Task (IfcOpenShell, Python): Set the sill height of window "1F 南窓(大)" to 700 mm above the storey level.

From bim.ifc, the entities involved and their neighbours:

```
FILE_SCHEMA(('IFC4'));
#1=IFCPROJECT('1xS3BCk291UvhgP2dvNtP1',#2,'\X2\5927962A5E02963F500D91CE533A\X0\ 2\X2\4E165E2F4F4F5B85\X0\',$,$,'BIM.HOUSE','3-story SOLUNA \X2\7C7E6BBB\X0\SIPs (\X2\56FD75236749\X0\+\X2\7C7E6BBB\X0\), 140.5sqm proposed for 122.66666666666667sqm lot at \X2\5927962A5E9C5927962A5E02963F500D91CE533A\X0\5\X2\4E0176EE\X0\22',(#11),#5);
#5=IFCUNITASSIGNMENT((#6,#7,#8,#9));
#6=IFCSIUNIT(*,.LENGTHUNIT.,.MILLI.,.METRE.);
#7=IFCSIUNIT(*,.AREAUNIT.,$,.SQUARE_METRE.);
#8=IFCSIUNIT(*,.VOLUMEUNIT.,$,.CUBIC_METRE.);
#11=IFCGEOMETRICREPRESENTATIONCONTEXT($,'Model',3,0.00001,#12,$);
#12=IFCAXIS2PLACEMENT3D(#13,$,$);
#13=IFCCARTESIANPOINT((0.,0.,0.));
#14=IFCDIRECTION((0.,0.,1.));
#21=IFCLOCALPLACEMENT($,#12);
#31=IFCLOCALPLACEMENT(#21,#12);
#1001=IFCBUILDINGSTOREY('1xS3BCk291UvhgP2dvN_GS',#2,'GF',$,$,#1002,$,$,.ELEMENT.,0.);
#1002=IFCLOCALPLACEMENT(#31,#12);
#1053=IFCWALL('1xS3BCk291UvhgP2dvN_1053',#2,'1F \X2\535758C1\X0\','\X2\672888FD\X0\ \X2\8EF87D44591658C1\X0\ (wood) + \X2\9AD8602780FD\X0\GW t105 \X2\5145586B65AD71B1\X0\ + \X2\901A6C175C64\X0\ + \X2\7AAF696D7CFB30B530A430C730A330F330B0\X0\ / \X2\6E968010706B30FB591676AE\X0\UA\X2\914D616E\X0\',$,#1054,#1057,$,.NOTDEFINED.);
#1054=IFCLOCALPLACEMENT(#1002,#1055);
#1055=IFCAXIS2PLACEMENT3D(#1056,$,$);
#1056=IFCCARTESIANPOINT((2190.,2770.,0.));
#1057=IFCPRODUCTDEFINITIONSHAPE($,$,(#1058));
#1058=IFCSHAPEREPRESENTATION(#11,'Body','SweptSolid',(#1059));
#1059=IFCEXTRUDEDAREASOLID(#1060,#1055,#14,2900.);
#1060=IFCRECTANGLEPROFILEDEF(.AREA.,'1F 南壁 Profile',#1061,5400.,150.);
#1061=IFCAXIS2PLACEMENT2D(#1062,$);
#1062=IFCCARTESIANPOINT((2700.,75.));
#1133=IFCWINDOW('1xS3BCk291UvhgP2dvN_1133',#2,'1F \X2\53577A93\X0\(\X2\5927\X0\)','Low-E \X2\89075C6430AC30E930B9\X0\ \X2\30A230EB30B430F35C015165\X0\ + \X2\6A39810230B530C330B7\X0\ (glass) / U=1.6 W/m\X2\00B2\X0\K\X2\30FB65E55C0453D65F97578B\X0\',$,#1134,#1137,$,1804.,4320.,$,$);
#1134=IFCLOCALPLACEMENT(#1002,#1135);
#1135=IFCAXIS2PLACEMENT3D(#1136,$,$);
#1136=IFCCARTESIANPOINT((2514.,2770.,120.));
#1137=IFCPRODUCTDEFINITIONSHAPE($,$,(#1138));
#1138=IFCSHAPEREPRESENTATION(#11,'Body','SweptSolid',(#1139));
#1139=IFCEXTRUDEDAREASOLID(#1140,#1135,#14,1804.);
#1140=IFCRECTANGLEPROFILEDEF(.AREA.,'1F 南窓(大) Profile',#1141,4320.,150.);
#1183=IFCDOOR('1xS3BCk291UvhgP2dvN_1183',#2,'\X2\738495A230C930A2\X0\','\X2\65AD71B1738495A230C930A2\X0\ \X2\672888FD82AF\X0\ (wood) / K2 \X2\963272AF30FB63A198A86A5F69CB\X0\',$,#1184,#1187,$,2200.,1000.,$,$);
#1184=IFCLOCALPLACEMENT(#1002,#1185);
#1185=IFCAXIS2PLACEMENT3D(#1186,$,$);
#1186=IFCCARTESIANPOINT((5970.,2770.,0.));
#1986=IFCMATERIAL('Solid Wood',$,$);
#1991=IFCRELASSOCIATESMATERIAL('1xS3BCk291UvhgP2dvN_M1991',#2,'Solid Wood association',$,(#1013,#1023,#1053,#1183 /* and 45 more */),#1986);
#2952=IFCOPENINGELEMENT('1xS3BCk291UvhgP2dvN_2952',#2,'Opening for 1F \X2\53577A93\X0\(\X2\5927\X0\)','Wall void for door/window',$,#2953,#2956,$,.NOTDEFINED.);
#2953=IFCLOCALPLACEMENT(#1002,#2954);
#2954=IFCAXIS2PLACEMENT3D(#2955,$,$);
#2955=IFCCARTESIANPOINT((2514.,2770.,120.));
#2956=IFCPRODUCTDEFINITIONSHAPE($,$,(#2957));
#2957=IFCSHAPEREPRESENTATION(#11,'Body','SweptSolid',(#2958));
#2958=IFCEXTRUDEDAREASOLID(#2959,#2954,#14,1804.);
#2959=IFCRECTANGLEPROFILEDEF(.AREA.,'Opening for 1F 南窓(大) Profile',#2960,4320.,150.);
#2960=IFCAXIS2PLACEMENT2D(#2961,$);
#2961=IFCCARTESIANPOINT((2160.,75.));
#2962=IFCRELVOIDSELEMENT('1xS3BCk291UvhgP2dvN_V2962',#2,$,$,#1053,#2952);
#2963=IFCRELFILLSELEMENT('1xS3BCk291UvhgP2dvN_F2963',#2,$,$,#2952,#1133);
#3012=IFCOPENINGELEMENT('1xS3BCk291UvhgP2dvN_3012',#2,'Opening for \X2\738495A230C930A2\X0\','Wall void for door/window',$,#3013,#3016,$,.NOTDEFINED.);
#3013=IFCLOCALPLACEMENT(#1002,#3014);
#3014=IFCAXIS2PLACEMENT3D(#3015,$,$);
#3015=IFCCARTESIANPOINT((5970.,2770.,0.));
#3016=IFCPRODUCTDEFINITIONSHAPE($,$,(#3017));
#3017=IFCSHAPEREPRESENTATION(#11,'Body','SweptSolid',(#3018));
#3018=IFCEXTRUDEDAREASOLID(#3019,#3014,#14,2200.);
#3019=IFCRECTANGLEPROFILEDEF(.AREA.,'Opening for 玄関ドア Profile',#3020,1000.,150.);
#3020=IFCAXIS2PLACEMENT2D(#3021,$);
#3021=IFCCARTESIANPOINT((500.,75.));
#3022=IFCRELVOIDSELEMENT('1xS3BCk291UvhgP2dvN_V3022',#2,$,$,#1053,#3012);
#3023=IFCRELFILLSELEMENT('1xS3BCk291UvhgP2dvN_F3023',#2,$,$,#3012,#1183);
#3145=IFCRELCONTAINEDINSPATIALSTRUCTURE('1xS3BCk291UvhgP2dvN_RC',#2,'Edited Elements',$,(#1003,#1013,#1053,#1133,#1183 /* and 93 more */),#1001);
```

```python
import numpy as np
import ifcopenshell
import ifcopenshell.api.geometry
import ifcopenshell.geom
import ifcopenshell.util.element
import ifcopenshell.util.placement
import ifcopenshell.util.shape
import ifcopenshell.util.unit

model = ifcopenshell.open("bim.ifc")
unit_scale = ifcopenshell.util.unit.calculate_unit_scale(model)

window = model.by_guid("1xS3BCk291UvhgP2dvN_1133")
opening = window.FillsVoids[0].RelatingOpeningElement
storey = ifcopenshell.util.element.get_container(window, ifc_class="IfcBuildingStorey")
level = ifcopenshell.util.placement.get_local_placement(storey.ObjectPlacement)[2, 3]

# The opening's origin need not be at the sill, so measure its lowest point.
shape = ifcopenshell.geom.create_shape(ifcopenshell.geom.settings(), opening)
bottom = ifcopenshell.util.shape.get_shape_bottom_elevation(shape, shape.geometry) / unit_scale
dz = level + 0.7 / unit_scale - bottom

shift = np.array([0.0, 0.0, dz])
# The window is not placed relative to its opening, so move both.
for product in (opening, window):
    matrix = ifcopenshell.util.placement.get_local_placement(product.ObjectPlacement)
    matrix[:3, 3] += shift
    ifcopenshell.api.geometry.edit_object_placement(model, product=product, matrix=matrix, is_si=False)

print(f"moved by {dz * unit_scale:+.3f} m")

model.write("bim-out.ifc")
```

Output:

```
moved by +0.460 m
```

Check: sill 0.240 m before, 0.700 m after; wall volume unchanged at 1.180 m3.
